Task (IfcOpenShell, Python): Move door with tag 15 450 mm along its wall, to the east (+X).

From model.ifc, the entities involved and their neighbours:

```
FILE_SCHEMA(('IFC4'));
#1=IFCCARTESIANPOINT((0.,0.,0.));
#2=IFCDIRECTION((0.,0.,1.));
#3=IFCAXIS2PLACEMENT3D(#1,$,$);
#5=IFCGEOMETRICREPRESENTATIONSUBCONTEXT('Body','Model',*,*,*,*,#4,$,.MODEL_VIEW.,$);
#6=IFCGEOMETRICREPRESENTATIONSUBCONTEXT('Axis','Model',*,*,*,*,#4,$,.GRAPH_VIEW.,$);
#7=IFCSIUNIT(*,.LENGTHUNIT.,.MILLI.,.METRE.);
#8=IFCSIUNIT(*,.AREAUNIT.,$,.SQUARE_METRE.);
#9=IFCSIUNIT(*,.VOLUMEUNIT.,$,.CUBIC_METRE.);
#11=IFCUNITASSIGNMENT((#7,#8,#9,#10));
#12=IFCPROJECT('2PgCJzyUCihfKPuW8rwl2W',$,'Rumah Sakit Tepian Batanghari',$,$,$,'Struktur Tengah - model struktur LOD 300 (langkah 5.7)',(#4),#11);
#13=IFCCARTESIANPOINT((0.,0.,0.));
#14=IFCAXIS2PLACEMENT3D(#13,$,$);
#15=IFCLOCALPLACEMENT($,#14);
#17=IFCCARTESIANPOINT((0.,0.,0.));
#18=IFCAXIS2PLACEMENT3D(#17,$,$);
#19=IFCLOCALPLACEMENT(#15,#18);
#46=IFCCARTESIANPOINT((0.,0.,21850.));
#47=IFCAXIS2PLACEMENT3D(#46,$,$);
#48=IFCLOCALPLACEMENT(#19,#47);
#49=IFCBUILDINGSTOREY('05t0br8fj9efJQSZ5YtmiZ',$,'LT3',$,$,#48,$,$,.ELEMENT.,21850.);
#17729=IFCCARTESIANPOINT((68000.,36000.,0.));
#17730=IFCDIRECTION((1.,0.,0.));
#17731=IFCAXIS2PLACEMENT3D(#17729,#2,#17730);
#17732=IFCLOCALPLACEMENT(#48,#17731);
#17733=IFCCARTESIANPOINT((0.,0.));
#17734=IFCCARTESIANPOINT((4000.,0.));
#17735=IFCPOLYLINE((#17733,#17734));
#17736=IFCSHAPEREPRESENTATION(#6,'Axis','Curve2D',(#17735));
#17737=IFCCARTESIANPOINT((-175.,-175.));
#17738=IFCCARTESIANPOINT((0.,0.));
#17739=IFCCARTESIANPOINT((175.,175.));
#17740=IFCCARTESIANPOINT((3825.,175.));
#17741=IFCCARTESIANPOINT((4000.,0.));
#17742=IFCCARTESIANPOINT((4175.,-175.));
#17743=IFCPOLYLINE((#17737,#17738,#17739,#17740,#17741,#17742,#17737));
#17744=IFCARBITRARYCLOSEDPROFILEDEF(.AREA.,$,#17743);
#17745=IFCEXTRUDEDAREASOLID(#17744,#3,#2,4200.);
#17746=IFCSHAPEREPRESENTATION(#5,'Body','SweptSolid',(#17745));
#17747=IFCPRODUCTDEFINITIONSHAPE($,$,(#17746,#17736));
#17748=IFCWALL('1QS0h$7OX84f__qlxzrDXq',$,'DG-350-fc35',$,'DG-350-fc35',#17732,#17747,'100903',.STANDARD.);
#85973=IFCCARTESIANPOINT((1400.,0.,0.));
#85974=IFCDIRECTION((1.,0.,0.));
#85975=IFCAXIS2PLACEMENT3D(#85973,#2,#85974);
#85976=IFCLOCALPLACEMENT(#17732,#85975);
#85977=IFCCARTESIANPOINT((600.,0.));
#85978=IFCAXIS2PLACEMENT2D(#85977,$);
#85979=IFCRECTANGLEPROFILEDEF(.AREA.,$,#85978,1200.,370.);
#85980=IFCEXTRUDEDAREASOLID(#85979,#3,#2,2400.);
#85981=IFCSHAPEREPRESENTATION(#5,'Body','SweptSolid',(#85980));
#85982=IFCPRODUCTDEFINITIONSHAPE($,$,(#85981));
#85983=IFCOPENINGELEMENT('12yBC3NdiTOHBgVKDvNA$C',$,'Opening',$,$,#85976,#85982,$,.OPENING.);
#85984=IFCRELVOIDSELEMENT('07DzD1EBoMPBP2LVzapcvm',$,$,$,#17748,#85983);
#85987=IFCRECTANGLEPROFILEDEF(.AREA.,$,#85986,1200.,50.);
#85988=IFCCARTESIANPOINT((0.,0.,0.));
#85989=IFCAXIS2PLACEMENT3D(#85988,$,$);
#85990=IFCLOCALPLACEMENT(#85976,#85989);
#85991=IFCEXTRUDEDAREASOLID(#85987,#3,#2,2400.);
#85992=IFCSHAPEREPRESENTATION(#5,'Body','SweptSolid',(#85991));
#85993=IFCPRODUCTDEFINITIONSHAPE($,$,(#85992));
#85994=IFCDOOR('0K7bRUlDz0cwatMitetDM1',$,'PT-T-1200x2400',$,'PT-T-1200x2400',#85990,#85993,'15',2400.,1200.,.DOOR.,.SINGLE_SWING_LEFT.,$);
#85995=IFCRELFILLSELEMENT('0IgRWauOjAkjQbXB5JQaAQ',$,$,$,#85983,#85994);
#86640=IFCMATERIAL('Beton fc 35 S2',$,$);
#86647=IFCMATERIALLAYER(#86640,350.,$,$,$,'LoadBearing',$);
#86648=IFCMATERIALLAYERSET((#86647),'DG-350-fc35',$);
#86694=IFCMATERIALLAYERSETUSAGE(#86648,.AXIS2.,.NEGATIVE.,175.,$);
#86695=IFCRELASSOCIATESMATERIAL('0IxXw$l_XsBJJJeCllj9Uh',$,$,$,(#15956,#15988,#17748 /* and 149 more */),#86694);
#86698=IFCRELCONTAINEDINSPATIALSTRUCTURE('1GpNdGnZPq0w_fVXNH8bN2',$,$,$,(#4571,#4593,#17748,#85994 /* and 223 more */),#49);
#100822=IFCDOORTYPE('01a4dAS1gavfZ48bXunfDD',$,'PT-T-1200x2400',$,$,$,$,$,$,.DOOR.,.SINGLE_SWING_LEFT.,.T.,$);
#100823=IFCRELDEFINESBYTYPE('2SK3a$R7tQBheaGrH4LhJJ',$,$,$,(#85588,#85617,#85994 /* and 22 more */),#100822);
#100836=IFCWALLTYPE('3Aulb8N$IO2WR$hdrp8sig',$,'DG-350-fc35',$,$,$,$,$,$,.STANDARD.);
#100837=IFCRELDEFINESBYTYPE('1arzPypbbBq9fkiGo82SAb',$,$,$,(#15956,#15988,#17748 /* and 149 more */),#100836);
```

```python
import ifcopenshell
import ifcopenshell.api.geometry
import ifcopenshell.util.placement

model = ifcopenshell.open("model.ifc")

door = model.by_guid("0K7bRUlDz0cwatMitetDM1")
opening = door.FillsVoids[0].RelatingOpeningElement
wall = opening.VoidsElements[0].RelatingBuildingElement

wall_matrix = ifcopenshell.util.placement.get_local_placement(wall.ObjectPlacement)
shift = wall_matrix[:3, 0] * 450.0
before = ifcopenshell.util.placement.get_local_placement(door.ObjectPlacement)[:3, 3].copy()

# The door is placed relative to its opening, so it follows when the opening moves.
matrix = ifcopenshell.util.placement.get_local_placement(opening.ObjectPlacement)
matrix[:3, 3] += shift
ifcopenshell.api.geometry.edit_object_placement(
    model, product=opening, matrix=matrix, is_si=False, should_transform_children=True
)

after = ifcopenshell.util.placement.get_local_placement(door.ObjectPlacement)[:3, 3]
print("door moved by", (after - before).round(3) + 0.0)

model.write("model-out.ifc")
```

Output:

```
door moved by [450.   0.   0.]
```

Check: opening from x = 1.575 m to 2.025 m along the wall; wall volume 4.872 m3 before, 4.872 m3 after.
